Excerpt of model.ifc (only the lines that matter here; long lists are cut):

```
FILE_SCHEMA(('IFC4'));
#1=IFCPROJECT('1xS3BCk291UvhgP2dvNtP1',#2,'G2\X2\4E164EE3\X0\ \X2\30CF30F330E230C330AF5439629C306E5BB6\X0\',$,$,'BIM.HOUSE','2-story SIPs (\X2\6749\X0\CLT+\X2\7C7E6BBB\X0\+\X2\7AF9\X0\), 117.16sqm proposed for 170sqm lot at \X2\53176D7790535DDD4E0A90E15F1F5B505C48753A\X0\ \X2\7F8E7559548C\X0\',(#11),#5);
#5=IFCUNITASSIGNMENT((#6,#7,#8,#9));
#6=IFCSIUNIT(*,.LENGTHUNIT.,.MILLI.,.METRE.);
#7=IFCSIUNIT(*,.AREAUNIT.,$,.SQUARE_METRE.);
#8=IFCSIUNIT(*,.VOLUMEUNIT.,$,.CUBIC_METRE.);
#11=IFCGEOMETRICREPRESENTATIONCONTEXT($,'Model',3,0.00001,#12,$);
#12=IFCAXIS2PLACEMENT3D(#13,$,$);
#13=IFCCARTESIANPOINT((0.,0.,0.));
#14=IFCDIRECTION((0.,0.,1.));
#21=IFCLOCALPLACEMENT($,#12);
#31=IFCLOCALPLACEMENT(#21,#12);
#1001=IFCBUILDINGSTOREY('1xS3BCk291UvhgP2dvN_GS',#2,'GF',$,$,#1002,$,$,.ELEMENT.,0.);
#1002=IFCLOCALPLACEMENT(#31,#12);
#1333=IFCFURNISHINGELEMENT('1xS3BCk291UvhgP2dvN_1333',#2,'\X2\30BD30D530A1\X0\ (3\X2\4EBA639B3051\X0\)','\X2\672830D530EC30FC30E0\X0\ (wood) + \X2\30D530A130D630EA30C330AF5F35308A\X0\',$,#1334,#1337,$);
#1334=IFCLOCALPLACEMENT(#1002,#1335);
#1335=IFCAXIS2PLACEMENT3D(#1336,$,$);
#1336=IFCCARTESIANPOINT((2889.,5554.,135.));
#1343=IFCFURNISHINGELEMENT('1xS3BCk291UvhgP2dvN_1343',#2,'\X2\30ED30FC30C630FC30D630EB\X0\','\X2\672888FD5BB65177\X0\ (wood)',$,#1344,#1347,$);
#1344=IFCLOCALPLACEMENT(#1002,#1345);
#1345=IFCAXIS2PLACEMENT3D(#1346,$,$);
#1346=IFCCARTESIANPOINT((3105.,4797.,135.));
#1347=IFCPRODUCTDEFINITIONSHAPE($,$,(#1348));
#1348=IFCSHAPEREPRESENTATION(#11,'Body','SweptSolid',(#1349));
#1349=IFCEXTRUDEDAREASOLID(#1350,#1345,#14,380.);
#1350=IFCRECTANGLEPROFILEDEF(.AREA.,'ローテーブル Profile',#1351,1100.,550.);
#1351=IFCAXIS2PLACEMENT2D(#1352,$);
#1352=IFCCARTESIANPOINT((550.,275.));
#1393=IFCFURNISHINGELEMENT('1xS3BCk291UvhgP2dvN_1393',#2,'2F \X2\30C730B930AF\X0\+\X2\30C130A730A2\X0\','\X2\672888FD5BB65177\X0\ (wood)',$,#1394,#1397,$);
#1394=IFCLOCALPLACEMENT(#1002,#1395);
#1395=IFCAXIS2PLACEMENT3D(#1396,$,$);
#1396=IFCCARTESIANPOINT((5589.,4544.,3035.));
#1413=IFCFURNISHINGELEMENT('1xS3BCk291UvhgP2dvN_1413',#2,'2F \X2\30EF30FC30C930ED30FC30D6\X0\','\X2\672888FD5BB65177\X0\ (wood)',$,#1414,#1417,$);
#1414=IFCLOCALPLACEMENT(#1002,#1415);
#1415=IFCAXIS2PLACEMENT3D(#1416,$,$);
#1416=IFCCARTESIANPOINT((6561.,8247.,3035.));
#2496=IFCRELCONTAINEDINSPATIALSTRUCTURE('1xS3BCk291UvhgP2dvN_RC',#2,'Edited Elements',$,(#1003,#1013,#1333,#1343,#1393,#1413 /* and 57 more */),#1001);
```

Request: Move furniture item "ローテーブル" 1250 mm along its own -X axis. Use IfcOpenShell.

```python
import ifcopenshell
import ifcopenshell.api.geometry
import ifcopenshell.util.placement
import ifcopenshell.util.unit

model = ifcopenshell.open("model.ifc")
unit_scale = ifcopenshell.util.unit.calculate_unit_scale(model)

item = model.by_guid("1xS3BCk291UvhgP2dvN_1343")
matrix = ifcopenshell.util.placement.get_local_placement(item.ObjectPlacement)
matrix[:3, 3] -= matrix[:3, 0] * 1.25 / unit_scale
ifcopenshell.api.geometry.edit_object_placement(model, product=item, matrix=matrix, is_si=False)

print(ifcopenshell.util.placement.get_local_placement(item.ObjectPlacement).round(3) + 0.0)

model.write("model_edited.ifc")
```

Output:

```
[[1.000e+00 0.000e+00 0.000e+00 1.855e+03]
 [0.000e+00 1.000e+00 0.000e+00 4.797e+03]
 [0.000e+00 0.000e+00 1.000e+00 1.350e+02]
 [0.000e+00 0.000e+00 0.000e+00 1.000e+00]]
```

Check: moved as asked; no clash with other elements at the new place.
